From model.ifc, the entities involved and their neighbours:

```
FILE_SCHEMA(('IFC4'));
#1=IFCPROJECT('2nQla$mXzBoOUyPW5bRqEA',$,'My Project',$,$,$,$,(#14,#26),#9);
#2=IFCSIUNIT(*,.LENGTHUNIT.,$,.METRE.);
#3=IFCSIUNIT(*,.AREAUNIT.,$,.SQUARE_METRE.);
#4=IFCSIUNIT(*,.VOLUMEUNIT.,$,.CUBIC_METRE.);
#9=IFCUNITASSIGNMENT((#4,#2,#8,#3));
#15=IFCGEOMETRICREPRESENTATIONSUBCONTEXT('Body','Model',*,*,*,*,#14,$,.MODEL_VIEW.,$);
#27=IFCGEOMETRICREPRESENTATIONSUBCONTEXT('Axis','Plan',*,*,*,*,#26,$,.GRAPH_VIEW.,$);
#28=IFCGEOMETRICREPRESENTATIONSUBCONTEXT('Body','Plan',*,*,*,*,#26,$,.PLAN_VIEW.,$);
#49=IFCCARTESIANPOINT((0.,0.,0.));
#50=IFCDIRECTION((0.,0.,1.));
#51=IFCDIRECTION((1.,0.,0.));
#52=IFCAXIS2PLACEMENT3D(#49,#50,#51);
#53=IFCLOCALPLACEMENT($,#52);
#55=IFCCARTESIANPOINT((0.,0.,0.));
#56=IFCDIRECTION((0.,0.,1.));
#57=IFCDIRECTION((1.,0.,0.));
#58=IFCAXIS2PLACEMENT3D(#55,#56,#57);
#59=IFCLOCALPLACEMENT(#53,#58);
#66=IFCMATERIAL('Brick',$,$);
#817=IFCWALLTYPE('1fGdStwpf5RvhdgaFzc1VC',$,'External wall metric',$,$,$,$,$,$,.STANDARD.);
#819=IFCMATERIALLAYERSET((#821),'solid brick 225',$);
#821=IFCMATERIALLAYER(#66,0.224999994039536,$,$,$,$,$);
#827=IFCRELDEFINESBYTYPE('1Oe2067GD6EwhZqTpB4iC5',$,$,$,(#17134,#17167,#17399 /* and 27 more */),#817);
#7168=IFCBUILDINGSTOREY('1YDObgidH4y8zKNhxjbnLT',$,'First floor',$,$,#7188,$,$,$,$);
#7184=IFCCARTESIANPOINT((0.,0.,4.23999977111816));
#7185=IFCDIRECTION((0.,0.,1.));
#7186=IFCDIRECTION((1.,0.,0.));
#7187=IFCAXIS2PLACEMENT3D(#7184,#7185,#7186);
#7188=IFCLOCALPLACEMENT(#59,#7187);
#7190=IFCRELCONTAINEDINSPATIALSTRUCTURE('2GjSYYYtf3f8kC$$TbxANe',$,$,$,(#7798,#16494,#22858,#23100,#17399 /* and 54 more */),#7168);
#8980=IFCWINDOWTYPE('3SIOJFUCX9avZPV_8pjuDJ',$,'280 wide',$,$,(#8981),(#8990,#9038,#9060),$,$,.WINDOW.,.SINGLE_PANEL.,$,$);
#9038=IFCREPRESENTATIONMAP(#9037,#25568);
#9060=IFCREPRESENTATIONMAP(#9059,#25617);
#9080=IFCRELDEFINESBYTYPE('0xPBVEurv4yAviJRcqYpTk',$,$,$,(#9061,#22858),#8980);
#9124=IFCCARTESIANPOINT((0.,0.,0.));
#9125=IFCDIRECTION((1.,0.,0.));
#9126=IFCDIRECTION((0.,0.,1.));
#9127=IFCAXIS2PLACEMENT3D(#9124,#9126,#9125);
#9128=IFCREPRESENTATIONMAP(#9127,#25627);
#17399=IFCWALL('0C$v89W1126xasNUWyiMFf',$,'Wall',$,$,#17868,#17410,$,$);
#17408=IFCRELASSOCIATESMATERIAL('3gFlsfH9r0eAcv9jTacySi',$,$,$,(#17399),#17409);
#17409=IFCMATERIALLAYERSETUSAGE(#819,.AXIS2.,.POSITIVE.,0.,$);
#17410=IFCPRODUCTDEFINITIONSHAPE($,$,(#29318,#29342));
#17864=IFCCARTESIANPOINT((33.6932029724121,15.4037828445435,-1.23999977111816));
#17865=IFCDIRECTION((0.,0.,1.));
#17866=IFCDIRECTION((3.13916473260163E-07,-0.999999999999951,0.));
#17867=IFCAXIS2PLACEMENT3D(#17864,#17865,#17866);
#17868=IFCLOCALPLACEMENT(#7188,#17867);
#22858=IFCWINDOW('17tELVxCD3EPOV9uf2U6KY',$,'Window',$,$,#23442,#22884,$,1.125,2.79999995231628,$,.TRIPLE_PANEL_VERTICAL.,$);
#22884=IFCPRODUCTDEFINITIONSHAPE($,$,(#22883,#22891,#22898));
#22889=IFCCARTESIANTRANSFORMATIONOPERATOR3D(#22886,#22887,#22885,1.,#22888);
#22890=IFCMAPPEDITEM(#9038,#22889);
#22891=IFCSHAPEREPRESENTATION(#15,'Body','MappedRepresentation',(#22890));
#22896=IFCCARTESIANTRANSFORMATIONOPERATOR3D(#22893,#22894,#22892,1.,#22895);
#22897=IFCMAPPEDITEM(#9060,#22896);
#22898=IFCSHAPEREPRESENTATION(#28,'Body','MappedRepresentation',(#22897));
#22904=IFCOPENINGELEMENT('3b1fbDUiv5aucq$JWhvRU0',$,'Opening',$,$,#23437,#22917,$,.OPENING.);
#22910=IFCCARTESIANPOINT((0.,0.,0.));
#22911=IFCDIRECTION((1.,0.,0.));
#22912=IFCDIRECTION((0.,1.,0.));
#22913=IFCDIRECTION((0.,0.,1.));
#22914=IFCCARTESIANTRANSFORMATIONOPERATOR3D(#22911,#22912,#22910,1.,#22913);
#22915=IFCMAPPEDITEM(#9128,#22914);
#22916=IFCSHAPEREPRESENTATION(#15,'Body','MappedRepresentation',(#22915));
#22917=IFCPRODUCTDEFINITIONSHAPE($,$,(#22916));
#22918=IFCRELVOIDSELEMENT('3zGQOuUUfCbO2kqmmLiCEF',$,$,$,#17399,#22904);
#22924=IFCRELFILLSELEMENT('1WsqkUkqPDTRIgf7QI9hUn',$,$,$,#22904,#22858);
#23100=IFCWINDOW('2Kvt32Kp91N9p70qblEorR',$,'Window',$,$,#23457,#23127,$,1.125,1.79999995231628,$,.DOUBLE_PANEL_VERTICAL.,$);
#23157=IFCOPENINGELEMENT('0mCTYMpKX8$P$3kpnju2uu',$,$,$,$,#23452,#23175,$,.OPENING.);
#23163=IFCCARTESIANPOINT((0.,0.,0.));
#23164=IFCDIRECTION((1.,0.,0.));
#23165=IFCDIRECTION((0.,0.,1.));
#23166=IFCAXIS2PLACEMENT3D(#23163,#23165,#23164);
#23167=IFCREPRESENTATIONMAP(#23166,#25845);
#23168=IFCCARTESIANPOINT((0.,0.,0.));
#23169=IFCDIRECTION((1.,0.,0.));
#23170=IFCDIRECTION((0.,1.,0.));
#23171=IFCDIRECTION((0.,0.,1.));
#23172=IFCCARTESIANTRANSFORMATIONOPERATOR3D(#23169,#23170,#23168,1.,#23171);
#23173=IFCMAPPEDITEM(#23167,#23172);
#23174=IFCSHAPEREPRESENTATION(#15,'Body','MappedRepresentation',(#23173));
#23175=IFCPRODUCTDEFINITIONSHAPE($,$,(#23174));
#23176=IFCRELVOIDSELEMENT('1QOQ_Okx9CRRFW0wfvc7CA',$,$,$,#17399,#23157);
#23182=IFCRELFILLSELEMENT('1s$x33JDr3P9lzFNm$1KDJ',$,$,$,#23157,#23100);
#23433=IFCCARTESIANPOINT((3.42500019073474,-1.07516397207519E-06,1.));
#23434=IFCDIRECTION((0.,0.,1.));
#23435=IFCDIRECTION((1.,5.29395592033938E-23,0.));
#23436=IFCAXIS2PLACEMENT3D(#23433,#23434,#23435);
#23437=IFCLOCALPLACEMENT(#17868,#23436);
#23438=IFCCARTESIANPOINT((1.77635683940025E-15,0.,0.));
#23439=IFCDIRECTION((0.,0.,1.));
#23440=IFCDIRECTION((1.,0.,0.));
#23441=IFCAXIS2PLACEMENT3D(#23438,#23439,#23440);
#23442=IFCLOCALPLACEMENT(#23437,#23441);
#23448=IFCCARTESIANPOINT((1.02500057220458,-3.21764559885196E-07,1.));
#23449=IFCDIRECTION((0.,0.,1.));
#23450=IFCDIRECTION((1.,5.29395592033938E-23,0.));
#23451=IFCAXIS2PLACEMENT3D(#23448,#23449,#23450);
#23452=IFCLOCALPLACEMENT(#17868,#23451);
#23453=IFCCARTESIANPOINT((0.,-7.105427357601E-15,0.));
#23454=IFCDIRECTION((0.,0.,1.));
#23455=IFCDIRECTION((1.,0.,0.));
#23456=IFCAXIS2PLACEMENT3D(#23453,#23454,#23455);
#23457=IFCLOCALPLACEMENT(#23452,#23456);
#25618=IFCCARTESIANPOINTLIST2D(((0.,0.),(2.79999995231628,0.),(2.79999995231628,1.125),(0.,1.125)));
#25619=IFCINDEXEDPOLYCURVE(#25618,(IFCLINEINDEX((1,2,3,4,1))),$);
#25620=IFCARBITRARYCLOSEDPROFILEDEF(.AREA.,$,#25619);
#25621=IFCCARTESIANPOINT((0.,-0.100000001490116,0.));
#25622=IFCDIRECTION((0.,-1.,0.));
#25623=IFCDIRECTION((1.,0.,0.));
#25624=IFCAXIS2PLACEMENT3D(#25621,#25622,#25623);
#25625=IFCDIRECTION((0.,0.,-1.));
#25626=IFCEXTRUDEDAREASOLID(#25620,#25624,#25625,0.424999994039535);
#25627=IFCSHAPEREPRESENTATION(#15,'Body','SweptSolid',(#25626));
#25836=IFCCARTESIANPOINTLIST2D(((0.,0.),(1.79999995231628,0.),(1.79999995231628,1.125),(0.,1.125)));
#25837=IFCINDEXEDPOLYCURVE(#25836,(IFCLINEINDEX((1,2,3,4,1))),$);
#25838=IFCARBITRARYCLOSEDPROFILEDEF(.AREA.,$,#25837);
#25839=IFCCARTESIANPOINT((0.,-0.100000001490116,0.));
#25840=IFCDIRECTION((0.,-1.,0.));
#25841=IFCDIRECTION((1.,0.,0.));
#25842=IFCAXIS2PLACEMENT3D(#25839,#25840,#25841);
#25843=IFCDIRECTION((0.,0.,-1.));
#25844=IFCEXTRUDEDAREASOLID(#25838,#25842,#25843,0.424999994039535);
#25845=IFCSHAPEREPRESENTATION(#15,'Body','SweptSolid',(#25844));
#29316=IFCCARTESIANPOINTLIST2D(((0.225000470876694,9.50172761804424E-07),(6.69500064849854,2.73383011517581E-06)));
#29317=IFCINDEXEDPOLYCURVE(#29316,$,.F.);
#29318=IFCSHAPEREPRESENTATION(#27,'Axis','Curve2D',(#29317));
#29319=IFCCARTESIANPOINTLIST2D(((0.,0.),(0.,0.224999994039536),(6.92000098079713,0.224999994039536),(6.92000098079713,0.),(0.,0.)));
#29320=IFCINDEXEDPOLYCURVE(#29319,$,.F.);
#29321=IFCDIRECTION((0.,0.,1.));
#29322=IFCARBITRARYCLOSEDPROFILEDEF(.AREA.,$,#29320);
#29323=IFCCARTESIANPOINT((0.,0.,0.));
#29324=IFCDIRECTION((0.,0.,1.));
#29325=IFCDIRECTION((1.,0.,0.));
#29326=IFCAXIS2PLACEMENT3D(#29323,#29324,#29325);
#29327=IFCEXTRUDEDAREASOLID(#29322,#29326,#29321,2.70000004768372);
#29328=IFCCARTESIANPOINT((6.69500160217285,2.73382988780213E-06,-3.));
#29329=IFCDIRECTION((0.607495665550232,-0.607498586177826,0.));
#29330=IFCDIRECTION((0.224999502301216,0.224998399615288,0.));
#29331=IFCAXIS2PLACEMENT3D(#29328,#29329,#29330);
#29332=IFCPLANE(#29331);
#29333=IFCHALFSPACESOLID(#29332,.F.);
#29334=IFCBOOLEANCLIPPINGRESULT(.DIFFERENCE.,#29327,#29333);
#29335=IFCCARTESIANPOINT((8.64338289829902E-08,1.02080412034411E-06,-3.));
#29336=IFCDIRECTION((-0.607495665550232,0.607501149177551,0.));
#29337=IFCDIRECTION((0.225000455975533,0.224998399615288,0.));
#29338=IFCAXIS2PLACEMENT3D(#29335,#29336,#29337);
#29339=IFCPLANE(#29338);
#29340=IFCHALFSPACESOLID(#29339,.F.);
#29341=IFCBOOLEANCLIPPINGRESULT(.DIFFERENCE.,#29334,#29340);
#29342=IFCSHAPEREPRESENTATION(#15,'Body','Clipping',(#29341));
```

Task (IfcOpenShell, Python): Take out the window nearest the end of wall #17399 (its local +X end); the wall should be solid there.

```python
import ifcopenshell
import ifcopenshell.api.feature
import ifcopenshell.api.root
import ifcopenshell.geom
import ifcopenshell.util.shape

model = ifcopenshell.open("model.ifc")
settings = ifcopenshell.geom.settings()


def volume(element):
    """Net volume in cubic metres, openings subtracted."""
    shape = ifcopenshell.geom.create_shape(settings, element)
    return ifcopenshell.util.shape.get_volume(shape.geometry)


window = model.by_guid("17tELVxCD3EPOV9uf2U6KY")
opening = window.FillsVoids[0].RelatingOpeningElement
wall = opening.VoidsElements[0].RelatingBuildingElement
before = volume(wall)

ifcopenshell.api.root.remove_product(model, product=window)
ifcopenshell.api.feature.remove_feature(model, feature=opening)

after = volume(wall)

print(f"wall volume {before:.3f} -> {after:.3f} m3")

model.write("model_v2.ifc")
```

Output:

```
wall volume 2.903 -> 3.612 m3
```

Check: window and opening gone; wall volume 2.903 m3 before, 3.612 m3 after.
